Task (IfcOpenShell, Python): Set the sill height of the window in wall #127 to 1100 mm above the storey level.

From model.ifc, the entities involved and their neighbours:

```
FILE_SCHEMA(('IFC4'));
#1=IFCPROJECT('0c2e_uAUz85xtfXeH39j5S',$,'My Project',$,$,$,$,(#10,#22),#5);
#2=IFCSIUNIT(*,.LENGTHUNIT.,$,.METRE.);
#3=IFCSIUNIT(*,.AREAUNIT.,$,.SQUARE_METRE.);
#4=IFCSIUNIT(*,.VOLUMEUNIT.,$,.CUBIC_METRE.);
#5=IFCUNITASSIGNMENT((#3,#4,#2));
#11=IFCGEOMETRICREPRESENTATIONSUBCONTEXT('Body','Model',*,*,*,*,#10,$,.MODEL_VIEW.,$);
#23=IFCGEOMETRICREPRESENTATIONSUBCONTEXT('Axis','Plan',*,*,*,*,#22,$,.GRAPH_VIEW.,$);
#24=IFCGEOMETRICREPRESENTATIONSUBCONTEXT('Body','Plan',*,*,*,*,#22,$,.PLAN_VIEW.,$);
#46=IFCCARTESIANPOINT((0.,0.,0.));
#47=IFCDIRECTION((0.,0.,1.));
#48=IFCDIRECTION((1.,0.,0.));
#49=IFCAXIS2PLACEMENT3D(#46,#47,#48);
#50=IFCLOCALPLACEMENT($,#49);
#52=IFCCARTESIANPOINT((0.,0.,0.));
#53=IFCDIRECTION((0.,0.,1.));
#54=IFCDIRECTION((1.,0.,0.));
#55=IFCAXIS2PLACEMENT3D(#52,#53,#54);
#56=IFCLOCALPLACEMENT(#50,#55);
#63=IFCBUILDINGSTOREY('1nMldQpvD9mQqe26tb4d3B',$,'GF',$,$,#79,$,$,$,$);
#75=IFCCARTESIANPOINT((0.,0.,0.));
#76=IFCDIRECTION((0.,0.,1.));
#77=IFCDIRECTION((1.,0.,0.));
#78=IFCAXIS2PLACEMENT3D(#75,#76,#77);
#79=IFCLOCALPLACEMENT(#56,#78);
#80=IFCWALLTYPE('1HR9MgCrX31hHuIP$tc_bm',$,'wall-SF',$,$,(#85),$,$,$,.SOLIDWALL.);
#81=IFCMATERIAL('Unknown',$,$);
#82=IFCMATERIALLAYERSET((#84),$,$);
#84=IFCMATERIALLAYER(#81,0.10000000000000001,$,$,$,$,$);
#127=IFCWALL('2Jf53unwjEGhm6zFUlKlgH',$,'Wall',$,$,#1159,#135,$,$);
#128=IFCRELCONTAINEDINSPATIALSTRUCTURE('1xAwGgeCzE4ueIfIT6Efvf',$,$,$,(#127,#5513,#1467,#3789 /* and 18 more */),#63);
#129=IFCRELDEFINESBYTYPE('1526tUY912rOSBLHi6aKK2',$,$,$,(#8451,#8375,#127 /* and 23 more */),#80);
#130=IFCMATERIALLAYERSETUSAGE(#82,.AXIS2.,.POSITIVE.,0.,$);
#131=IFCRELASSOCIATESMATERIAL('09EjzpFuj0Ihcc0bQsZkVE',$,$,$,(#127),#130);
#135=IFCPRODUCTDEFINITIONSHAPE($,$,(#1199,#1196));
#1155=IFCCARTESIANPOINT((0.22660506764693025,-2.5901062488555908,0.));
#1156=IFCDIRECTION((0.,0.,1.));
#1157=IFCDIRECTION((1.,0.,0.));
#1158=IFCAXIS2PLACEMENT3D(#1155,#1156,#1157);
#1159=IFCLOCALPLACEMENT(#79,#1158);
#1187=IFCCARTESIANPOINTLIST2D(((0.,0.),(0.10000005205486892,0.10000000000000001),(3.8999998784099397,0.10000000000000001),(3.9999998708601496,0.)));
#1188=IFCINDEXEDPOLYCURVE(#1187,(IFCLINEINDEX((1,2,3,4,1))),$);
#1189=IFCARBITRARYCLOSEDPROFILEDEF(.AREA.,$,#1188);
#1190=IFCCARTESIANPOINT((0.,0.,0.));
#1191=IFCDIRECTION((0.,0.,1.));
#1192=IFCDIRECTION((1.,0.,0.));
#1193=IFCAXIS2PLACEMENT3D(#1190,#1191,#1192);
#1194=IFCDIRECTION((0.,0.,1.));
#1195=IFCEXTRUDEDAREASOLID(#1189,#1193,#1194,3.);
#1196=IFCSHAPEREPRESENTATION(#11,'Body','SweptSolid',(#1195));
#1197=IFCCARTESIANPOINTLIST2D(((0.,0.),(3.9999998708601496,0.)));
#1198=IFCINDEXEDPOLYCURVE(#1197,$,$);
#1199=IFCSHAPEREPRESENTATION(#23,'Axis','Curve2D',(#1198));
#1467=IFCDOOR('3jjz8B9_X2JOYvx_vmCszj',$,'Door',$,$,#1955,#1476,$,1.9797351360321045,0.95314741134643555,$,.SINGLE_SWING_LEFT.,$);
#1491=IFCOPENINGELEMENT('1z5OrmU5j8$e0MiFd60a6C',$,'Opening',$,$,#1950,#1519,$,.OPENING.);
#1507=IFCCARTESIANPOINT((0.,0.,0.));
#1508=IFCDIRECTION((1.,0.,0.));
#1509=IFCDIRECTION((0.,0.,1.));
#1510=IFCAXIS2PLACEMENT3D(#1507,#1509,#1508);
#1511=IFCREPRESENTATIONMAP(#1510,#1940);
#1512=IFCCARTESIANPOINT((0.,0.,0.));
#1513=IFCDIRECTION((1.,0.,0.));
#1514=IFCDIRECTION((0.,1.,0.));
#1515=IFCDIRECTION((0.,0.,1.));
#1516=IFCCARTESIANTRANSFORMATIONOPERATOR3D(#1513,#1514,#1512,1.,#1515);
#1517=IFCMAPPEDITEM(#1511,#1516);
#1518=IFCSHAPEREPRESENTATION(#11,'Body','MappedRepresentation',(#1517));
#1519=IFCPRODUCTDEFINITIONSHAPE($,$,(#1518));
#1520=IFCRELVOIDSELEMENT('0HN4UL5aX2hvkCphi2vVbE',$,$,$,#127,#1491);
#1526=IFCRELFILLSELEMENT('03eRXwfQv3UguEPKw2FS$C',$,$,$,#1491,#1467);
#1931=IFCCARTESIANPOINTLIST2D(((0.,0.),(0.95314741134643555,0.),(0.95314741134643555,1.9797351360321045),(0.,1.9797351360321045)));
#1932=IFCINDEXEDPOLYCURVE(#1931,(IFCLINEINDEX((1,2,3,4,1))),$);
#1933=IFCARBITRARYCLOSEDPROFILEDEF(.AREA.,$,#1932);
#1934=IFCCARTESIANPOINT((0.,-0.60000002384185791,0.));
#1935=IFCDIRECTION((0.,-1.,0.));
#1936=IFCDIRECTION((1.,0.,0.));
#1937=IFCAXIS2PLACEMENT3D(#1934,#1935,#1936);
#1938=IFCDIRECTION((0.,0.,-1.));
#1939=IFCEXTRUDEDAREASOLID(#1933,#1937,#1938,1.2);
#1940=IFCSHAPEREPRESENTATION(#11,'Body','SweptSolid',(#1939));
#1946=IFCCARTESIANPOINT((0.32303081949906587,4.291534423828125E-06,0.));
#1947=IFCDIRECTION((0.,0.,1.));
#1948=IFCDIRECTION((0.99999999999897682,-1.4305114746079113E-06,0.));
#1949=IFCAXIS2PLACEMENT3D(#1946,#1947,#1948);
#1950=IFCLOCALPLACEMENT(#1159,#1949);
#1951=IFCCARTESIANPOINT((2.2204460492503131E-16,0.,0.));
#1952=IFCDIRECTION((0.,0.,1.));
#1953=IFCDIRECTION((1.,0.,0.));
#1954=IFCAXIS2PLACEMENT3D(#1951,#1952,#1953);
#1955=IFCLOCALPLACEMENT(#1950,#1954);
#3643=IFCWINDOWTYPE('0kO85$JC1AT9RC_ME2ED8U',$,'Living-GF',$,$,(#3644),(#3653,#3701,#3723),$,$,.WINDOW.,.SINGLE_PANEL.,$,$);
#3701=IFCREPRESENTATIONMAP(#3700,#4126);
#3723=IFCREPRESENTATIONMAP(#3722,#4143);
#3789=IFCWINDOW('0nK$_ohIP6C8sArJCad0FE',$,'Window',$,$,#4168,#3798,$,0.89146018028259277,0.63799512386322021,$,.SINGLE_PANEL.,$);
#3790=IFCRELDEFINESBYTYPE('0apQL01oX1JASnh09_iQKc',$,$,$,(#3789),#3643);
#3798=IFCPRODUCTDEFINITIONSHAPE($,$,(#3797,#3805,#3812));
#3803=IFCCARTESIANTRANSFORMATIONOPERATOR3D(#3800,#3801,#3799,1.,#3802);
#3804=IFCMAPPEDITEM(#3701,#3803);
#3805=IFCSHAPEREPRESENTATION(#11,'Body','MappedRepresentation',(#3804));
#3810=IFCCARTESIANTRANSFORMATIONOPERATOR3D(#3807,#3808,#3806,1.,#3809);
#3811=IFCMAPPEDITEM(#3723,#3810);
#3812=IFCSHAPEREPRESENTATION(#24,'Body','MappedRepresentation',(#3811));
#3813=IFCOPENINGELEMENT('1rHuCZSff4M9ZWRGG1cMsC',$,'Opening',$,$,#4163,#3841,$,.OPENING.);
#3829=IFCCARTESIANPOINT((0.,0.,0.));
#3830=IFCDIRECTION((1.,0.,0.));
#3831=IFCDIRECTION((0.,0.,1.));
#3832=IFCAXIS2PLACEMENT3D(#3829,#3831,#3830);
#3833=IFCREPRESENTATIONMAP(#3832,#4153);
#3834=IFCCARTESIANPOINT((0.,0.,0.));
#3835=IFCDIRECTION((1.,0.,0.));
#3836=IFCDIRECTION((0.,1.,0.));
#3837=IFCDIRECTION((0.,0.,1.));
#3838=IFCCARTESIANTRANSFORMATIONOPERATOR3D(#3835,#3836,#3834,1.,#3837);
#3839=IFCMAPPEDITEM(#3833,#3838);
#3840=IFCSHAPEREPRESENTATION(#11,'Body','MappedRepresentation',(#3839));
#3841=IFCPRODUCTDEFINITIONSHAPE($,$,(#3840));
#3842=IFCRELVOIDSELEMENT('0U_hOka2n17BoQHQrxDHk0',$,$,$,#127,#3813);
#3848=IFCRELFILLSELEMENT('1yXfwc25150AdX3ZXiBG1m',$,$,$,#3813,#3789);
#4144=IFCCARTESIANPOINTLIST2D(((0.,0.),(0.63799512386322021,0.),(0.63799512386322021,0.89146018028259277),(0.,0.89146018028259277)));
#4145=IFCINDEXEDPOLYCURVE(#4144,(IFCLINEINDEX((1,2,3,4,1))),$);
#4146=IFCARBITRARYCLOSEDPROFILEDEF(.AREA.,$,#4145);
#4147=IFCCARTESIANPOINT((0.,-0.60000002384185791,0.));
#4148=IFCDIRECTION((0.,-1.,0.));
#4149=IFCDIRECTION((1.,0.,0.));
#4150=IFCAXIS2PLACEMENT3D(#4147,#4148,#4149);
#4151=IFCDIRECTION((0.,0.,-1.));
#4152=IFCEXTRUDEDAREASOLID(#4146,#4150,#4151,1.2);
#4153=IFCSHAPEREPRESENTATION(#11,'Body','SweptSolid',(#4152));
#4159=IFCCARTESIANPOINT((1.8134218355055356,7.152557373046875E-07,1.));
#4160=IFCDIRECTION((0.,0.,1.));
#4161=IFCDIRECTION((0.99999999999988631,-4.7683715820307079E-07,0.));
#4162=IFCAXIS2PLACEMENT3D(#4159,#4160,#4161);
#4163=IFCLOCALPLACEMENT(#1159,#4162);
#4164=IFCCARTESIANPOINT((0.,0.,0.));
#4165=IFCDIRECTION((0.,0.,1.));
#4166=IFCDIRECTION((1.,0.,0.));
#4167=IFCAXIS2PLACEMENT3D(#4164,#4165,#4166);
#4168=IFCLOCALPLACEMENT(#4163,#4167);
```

```python
import numpy as np
import ifcopenshell
import ifcopenshell.api.geometry
import ifcopenshell.geom
import ifcopenshell.util.element
import ifcopenshell.util.placement
import ifcopenshell.util.shape
import ifcopenshell.util.unit

model = ifcopenshell.open("model.ifc")
unit_scale = ifcopenshell.util.unit.calculate_unit_scale(model)

window = model.by_guid("0nK$_ohIP6C8sArJCad0FE")
opening = window.FillsVoids[0].RelatingOpeningElement
storey = ifcopenshell.util.element.get_container(window, ifc_class="IfcBuildingStorey")
level = ifcopenshell.util.placement.get_local_placement(storey.ObjectPlacement)[2, 3]

# The opening's origin need not be at the sill, so measure its lowest point.
shape = ifcopenshell.geom.create_shape(ifcopenshell.geom.settings(), opening)
bottom = ifcopenshell.util.shape.get_shape_bottom_elevation(shape, shape.geometry) / unit_scale
dz = level + 1.1 / unit_scale - bottom

shift = np.array([0.0, 0.0, dz])
# The window is placed relative to its opening, so it follows when the opening moves.
matrix = ifcopenshell.util.placement.get_local_placement(opening.ObjectPlacement)
matrix[:3, 3] += shift
ifcopenshell.api.geometry.edit_object_placement(
    model, product=opening, matrix=matrix, is_si=False, should_transform_children=True
)

print(f"moved by {dz * unit_scale:+.3f} m")

model.write("model_rev.ifc")
```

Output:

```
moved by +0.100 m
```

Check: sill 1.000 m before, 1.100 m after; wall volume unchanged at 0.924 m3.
